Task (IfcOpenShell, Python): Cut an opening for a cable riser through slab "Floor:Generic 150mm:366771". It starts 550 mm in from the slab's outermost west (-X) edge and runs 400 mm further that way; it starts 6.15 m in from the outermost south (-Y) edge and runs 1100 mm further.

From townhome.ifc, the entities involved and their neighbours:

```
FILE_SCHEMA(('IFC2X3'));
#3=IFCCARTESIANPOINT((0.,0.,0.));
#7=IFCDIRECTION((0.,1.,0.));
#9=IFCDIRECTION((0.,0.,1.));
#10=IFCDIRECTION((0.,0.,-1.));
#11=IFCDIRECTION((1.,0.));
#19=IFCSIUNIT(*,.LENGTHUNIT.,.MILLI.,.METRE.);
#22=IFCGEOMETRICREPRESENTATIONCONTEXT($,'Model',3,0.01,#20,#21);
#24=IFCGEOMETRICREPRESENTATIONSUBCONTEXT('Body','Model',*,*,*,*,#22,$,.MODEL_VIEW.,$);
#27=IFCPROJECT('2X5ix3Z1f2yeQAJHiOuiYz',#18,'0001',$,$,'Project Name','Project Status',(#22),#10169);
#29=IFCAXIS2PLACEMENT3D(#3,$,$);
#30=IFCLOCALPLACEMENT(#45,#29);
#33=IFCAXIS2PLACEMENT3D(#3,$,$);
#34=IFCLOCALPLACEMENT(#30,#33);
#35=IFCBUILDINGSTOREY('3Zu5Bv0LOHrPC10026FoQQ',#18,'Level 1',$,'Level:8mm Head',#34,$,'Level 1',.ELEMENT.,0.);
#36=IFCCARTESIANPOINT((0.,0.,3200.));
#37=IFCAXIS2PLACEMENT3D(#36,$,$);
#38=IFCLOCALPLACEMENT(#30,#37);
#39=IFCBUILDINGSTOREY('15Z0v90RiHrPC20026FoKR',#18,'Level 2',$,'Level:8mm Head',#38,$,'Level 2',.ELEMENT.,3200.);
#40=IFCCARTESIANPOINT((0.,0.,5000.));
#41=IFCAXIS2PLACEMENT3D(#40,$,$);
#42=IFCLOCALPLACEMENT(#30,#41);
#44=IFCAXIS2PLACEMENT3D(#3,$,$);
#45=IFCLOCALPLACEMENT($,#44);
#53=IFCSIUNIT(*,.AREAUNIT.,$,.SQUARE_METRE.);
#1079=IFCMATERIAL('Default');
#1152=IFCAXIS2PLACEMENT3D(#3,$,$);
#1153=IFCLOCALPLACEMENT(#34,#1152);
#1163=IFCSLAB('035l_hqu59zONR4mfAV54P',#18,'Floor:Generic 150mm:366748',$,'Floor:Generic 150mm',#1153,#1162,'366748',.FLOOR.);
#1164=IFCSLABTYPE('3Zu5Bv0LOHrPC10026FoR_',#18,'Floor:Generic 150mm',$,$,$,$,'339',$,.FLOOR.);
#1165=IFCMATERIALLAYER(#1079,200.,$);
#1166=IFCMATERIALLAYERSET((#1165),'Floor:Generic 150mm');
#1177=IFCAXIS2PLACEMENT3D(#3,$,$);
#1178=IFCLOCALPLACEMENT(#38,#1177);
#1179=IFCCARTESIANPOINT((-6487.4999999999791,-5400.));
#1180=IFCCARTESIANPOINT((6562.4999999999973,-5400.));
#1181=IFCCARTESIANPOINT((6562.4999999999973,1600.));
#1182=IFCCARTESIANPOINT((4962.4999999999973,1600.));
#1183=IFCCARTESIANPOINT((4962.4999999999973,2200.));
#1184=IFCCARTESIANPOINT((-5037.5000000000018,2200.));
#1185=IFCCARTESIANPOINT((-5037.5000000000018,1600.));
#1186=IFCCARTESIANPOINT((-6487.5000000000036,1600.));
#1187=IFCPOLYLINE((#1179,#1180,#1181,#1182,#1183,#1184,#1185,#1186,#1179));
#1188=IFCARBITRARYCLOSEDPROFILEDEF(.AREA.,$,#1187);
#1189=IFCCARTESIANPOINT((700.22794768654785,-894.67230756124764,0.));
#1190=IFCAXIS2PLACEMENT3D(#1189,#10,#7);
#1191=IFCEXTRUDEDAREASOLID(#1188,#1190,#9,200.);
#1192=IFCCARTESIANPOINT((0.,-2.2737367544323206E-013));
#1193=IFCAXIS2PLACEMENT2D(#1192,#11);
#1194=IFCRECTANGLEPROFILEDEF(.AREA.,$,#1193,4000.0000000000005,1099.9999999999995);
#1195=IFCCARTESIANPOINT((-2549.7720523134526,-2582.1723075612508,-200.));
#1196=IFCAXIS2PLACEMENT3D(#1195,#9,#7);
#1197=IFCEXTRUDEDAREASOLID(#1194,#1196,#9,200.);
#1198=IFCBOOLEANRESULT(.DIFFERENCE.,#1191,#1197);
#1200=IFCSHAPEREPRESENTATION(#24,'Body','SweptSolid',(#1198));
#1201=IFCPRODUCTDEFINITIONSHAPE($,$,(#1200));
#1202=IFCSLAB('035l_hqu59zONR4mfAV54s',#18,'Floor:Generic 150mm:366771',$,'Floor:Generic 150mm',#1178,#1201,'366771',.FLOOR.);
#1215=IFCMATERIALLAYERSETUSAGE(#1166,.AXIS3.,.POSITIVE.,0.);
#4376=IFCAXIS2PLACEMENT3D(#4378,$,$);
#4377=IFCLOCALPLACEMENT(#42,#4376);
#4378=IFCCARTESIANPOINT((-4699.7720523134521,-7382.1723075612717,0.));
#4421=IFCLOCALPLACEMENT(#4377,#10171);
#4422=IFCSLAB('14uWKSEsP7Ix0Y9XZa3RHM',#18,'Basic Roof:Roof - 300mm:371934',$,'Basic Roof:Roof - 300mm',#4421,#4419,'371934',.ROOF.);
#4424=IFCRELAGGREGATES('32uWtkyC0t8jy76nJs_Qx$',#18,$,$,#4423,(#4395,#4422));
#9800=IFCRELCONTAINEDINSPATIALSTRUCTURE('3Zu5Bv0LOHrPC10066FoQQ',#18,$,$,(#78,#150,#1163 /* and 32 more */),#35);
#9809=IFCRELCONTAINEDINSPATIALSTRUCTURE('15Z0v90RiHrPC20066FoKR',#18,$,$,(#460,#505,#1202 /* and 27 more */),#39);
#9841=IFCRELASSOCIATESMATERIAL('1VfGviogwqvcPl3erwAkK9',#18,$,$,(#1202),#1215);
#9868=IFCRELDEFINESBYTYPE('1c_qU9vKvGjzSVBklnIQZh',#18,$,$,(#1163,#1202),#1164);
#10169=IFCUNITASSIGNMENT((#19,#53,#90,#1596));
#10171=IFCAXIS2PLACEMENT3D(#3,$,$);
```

```python
import numpy as np
import ifcopenshell
import ifcopenshell.api.feature
import ifcopenshell.api.geometry
import ifcopenshell.api.root
import ifcopenshell.geom
import ifcopenshell.util.placement
import ifcopenshell.util.representation
import ifcopenshell.util.shape
import ifcopenshell.util.unit

model = ifcopenshell.open("townhome.ifc")
unit_scale = ifcopenshell.util.unit.calculate_unit_scale(model)
settings = ifcopenshell.geom.settings()


def volume(element):
    """Net volume in cubic metres, openings subtracted."""
    shape = ifcopenshell.geom.create_shape(settings, element)
    return ifcopenshell.util.shape.get_volume(shape.geometry)


slab = model.by_id(1202)
before = volume(slab)

# Extent in the slab's own axes, in metres. The edges named are its -X and -Y sides.
slab_shape = ifcopenshell.geom.create_shape(settings, slab)
vertices = ifcopenshell.util.shape.get_vertices(slab_shape.geometry)
x_min, y_min, bottom = vertices.min(axis=0)
top = vertices[:, 2].max()

opening = ifcopenshell.api.root.create_entity(model, ifc_class="IfcOpeningElement", name="Cable riser opening")
context = ifcopenshell.util.representation.get_context(model, "Model", "Body", "MODEL_VIEW")
width, depth = 0.4, 1.1
outline = [(0.0, 0.0), (width, 0.0), (width, depth), (0.0, depth), (0.0, 0.0)]
# Overshoot both faces by 50 mm so the cut is clean.
shape = ifcopenshell.api.geometry.add_slab_representation(
    model, context=context, depth=top - bottom + 0.1, polyline=outline
)
ifcopenshell.api.geometry.assign_representation(model, product=opening, representation=shape)

matrix = ifcopenshell.util.placement.get_local_placement(slab.ObjectPlacement)
matrix[:, 3] = matrix @ np.append(np.array([x_min + 0.55, y_min + 6.15, bottom - 0.05]) / unit_scale, 1.0)
ifcopenshell.api.geometry.edit_object_placement(model, product=opening, matrix=matrix, is_si=False)
ifcopenshell.api.feature.add_feature(model, feature=opening, element=slab)

after = volume(slab)

print(f"slab volume {before:.3f} -> {after:.3f} m3")

model.write("townhome_edited.ifc")
```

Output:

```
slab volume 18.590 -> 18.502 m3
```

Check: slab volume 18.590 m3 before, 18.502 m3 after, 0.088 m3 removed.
